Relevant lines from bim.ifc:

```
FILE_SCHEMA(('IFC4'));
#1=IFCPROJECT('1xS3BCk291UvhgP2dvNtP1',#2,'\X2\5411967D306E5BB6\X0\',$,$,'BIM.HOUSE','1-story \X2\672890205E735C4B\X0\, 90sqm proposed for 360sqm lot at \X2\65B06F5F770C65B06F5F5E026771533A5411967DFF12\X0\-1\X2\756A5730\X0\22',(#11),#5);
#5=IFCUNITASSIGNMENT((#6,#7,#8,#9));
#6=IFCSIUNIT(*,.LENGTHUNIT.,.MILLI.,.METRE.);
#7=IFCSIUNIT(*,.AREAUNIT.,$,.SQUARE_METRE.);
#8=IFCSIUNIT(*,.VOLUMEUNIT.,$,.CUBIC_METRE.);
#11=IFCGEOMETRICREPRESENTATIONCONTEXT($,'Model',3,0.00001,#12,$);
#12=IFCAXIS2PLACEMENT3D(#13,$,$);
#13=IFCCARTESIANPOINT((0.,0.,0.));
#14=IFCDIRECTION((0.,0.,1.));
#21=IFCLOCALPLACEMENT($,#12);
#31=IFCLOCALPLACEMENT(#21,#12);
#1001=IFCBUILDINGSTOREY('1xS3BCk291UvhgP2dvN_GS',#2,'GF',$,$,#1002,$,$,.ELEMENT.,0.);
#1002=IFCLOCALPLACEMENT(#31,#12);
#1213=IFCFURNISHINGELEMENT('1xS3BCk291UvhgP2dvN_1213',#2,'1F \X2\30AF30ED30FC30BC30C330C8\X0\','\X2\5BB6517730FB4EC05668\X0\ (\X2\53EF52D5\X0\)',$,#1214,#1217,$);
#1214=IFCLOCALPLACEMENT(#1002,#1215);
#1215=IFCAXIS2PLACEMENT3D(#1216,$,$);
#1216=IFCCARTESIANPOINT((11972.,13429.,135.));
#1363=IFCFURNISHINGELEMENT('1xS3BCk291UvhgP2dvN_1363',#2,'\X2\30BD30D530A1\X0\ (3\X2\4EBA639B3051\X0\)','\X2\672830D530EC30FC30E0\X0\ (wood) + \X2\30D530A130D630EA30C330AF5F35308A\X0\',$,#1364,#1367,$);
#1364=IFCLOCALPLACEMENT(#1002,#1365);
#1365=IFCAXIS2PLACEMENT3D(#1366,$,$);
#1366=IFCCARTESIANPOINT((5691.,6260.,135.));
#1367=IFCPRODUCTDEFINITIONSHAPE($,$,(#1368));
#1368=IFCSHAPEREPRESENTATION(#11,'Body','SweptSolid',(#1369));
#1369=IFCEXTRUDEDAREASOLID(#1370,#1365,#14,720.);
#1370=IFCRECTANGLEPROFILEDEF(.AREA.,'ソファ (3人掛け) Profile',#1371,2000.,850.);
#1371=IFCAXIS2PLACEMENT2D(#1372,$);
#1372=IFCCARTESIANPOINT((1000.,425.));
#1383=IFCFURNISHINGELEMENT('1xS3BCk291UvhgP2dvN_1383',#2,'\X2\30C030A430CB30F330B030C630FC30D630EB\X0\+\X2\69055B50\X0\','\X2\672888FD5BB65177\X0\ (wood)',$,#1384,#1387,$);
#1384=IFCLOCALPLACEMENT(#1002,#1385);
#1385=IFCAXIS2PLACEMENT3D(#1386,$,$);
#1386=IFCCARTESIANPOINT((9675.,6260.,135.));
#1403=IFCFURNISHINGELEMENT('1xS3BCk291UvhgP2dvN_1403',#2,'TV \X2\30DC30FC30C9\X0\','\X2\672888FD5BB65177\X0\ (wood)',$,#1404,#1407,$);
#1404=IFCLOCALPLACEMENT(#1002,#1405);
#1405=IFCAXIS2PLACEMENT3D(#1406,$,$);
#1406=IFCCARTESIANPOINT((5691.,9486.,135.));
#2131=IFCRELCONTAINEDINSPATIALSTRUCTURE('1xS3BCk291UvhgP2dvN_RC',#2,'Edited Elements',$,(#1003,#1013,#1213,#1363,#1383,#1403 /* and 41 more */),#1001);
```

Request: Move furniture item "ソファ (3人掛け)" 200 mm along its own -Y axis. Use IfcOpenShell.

```python
import ifcopenshell
import ifcopenshell.api.geometry
import ifcopenshell.util.placement
import ifcopenshell.util.unit

model = ifcopenshell.open("bim.ifc")
unit_scale = ifcopenshell.util.unit.calculate_unit_scale(model)

item = model.by_guid("1xS3BCk291UvhgP2dvN_1363")
matrix = ifcopenshell.util.placement.get_local_placement(item.ObjectPlacement)
matrix[:3, 3] -= matrix[:3, 1] * 0.2 / unit_scale
ifcopenshell.api.geometry.edit_object_placement(model, product=item, matrix=matrix, is_si=False)

print(ifcopenshell.util.placement.get_local_placement(item.ObjectPlacement).round(3) + 0.0)

model.write("bim_edited.ifc")
```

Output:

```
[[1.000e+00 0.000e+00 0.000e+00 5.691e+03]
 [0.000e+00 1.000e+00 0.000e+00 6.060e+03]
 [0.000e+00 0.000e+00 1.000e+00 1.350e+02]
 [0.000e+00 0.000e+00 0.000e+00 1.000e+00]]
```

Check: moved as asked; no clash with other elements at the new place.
